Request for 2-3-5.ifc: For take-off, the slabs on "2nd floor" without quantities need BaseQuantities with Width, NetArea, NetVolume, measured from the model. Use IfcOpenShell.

First a look at what the model holds.

```python
import ifcopenshell
import ifcopenshell.util.element
import ifcopenshell.util.unit

model = ifcopenshell.open("2-3-5.ifc")
print(model.schema)
for unit_type in ("LENGTHUNIT", "AREAUNIT", "VOLUMEUNIT"):
    print(unit_type, ifcopenshell.util.unit.calculate_unit_scale(model, unit_type))
storey = next(s for s in model.by_type("IfcBuildingStorey") if s.Name == "2nd floor")
slabs = [e for e in ifcopenshell.util.element.get_decomposition(storey) if e.is_a("IfcSlab")]
for e in sorted(slabs, key=lambda e: e.id()):
    print(e.id(), e.is_a(), e.Name, list(ifcopenshell.util.element.get_psets(e, qtos_only=True)), sep=" | ")
```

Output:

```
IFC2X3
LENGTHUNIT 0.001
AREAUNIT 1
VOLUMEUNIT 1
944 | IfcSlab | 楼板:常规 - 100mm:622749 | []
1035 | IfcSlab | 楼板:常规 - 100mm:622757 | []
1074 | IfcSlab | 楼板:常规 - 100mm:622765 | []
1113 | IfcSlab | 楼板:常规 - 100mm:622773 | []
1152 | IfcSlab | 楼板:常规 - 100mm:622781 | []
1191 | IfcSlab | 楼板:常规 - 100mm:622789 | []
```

```python
import ifcopenshell
import ifcopenshell.api.pset
import ifcopenshell.geom
import ifcopenshell.util.element
import ifcopenshell.util.shape
import ifcopenshell.util.unit

model = ifcopenshell.open("2-3-5.ifc")
unit_scale = ifcopenshell.util.unit.calculate_unit_scale(model)
area_scale = ifcopenshell.util.unit.calculate_unit_scale(model, "AREAUNIT")
volume_scale = ifcopenshell.util.unit.calculate_unit_scale(model, "VOLUMEUNIT")
settings = ifcopenshell.geom.settings()

storey = next(s for s in model.by_type("IfcBuildingStorey") if s.Name == "2nd floor")
slabs = [e for e in ifcopenshell.util.element.get_decomposition(storey) if e.is_a("IfcSlab")]

for e in sorted(slabs, key=lambda e: e.id()):
    if ifcopenshell.util.element.get_psets(e, qtos_only=True, should_inherit=False):
        continue
    # Geometry comes back in metres, in the element's own axes.
    shape = ifcopenshell.geom.create_shape(settings, e)
    values = {
        "Width": ifcopenshell.util.shape.get_z(shape.geometry) / unit_scale,
        "NetArea": ifcopenshell.util.shape.get_footprint_area(shape.geometry) / area_scale,
        "NetVolume": ifcopenshell.util.shape.get_volume(shape.geometry) / volume_scale,
    }
    qto = ifcopenshell.api.pset.add_qto(model, product=e, name="BaseQuantities")
    ifcopenshell.api.pset.edit_qto(model, qto=qto, properties=values)
    print(e.id(), {k: round(v, 3) for k, v in values.items()})

model.write("2-3-5_v2.ifc")
```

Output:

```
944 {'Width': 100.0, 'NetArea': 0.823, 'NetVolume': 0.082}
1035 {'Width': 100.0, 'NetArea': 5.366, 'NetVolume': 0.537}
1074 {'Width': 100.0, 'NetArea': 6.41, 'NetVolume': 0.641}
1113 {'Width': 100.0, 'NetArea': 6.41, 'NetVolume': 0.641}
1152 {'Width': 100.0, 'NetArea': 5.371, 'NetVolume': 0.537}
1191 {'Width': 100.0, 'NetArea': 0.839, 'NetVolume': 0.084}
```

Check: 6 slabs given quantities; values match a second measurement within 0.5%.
